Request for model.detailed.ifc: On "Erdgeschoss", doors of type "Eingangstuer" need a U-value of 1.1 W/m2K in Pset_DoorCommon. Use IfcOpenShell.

First a look at what the model holds.

```python
import ifcopenshell
import ifcopenshell.util.element

model = ifcopenshell.open("model.detailed.ifc")
print(model.schema)
storey = next(s for s in model.by_type("IfcBuildingStorey") if s.Name == "Erdgeschoss")
doors = [e for e in ifcopenshell.util.element.get_decomposition(storey) if e.is_a("IfcDoor")]
seen = {}
for e in doors:
    element_type = ifcopenshell.util.element.get_type(e)
    key = (element_type.Name if element_type != e and element_type else None, ifcopenshell.util.element.get_pset(e, "Pset_DoorCommon", "ThermalTransmittance"))
    seen[key] = seen.get(key, 0) + 1
for (name, value), count in sorted(seen.items(), key=str):
    print(count, "x", name, "|", value)
```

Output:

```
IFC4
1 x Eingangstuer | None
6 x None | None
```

```python
import ifcopenshell
import ifcopenshell.api.pset
import ifcopenshell.util.element

model = ifcopenshell.open("model.detailed.ifc")

storey = next(s for s in model.by_type("IfcBuildingStorey") if s.Name == "Erdgeschoss")
doors = [e for e in ifcopenshell.util.element.get_decomposition(storey) if e.is_a("IfcDoor")]

count = 0
for e in doors:
    element_type = ifcopenshell.util.element.get_type(e)
    if element_type in (None, e) or element_type.Name != "Eingangstuer":
        continue
    # add_pset returns the element's existing set when there is one.
    pset = ifcopenshell.api.pset.add_pset(model, product=e, name="Pset_DoorCommon")
    ifcopenshell.api.pset.edit_pset(model, pset=pset, properties={"ThermalTransmittance": 1.1})
    count += 1

print(count, "doors updated")

model.write("model.detailed_edited.ifc")
```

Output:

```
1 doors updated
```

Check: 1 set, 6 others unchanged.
